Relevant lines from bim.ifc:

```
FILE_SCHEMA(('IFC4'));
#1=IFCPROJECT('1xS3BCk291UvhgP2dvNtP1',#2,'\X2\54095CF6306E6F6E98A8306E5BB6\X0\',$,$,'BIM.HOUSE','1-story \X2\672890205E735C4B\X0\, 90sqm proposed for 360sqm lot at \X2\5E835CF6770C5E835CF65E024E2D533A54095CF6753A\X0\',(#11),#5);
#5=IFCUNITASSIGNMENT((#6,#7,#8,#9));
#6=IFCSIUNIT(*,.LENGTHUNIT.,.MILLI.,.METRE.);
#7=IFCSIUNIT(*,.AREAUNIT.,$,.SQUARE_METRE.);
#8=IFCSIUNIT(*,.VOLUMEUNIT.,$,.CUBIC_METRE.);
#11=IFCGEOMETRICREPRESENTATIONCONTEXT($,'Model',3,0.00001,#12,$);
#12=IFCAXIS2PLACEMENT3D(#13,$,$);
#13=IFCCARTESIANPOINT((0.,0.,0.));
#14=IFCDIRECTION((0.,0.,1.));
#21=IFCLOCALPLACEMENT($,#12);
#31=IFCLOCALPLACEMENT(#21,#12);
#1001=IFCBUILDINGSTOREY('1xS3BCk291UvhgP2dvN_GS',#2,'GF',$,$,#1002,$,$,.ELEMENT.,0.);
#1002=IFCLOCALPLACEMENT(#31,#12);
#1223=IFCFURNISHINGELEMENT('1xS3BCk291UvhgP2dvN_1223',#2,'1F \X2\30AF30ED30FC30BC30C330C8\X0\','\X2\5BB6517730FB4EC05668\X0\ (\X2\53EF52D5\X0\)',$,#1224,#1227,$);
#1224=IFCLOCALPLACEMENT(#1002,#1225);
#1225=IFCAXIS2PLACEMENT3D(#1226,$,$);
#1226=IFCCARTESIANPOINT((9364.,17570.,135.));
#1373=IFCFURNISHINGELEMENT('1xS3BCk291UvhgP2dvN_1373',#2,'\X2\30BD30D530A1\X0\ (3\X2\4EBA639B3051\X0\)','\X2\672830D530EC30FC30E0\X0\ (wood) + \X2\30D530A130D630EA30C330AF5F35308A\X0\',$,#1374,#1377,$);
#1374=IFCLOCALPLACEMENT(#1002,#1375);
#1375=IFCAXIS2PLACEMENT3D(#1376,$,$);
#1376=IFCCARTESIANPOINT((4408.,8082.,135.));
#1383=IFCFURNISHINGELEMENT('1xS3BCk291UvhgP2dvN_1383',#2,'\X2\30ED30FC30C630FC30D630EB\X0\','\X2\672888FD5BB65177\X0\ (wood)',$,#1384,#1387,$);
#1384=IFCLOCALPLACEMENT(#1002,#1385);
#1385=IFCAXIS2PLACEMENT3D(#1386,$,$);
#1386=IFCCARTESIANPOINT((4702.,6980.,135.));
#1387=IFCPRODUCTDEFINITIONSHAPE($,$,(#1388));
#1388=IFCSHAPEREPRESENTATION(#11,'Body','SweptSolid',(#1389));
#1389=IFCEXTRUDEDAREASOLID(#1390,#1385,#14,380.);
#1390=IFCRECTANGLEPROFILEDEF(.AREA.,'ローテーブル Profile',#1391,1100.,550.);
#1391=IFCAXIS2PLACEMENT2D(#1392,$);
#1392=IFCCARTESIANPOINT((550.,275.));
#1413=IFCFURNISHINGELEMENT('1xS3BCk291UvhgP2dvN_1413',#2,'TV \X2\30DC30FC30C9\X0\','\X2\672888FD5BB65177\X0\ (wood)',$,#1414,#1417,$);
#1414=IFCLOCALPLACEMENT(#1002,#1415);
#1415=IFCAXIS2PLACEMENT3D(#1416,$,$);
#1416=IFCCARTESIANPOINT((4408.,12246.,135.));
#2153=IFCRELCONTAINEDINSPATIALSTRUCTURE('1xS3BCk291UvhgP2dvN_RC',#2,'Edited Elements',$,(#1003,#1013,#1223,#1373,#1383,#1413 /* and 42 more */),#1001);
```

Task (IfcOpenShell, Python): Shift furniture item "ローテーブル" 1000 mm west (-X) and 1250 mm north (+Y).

```python
import ifcopenshell
import ifcopenshell.api.geometry
import ifcopenshell.util.placement
import ifcopenshell.util.unit

model = ifcopenshell.open("bim.ifc")
unit_scale = ifcopenshell.util.unit.calculate_unit_scale(model)

item = model.by_id(1383)
matrix = ifcopenshell.util.placement.get_local_placement(item.ObjectPlacement)
matrix[0, 3] -= 1 / unit_scale
matrix[1, 3] += 1.25 / unit_scale
ifcopenshell.api.geometry.edit_object_placement(model, product=item, matrix=matrix, is_si=False)

print(ifcopenshell.util.placement.get_local_placement(item.ObjectPlacement).round(3) + 0.0)

model.write("bim_updated.ifc")
```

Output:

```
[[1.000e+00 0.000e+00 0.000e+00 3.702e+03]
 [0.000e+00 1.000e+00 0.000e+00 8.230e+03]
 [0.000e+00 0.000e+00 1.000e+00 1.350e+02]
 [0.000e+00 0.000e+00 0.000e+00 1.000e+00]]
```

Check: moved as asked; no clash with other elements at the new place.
